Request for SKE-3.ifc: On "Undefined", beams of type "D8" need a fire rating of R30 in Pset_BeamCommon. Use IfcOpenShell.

First a look at what the model holds.

```python
import ifcopenshell
import ifcopenshell.util.element

model = ifcopenshell.open("SKE-3.ifc")
print(model.schema)
storey = next(s for s in model.by_type("IfcBuildingStorey") if s.Name == "Undefined")
beams = [e for e in ifcopenshell.util.element.get_decomposition(storey) if e.is_a("IfcBeam")]
seen = {}
for e in beams:
    element_type = ifcopenshell.util.element.get_type(e)
    key = (element_type.Name if element_type != e and element_type else None, ifcopenshell.util.element.get_pset(e, "Pset_BeamCommon", "FireRating"))
    seen[key] = seen.get(key, 0) + 1
for (name, value), count in sorted(seen.items(), key=str):
    print(count, "x", name, "|", value)
```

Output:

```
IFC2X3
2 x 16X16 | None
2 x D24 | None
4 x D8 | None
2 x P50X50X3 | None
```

```python
import ifcopenshell
import ifcopenshell.api.pset
import ifcopenshell.util.element

model = ifcopenshell.open("SKE-3.ifc")

storey = next(s for s in model.by_type("IfcBuildingStorey") if s.Name == "Undefined")
beams = [e for e in ifcopenshell.util.element.get_decomposition(storey) if e.is_a("IfcBeam")]

count = 0
for e in beams:
    element_type = ifcopenshell.util.element.get_type(e)
    if element_type in (None, e) or element_type.Name != "D8":
        continue
    found = ifcopenshell.util.element.get_pset(e, "Pset_BeamCommon", should_inherit=False)
    if found:
        pset = model.by_id(found["id"])
        if len(ifcopenshell.util.element.get_elements_by_pset(pset)) > 1:
            pset = ifcopenshell.api.pset.unshare_pset(model, products=[e], pset=pset)[0]
    else:
        pset = ifcopenshell.api.pset.add_pset(model, product=e, name="Pset_BeamCommon")
    ifcopenshell.api.pset.edit_pset(model, pset=pset, properties={"FireRating": "R30"})
    count += 1

print(count, "beams updated")

model.write("SKE-3_v2.ifc")
```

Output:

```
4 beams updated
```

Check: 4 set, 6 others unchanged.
